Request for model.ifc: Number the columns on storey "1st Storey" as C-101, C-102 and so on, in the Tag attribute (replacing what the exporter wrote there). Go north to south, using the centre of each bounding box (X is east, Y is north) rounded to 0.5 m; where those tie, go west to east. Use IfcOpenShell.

First a look at what the model holds.

```python
import ifcopenshell
import ifcopenshell.util.element
import ifcopenshell.util.placement

model = ifcopenshell.open("model.ifc")
print(model.schema)
storey = next(s for s in model.by_type("IfcBuildingStorey") if s.Name == "1st Storey")
columns = [e for e in ifcopenshell.util.element.get_decomposition(storey) if e.is_a("IfcColumn")]
for e in sorted(columns, key=lambda e: e.id()):
    origin = ifcopenshell.util.placement.get_local_placement(e.ObjectPlacement)[:3, 3]
    print(e.id(), e.Tag, e.Name, origin.round(2) + 0.0, sep=" | ")
```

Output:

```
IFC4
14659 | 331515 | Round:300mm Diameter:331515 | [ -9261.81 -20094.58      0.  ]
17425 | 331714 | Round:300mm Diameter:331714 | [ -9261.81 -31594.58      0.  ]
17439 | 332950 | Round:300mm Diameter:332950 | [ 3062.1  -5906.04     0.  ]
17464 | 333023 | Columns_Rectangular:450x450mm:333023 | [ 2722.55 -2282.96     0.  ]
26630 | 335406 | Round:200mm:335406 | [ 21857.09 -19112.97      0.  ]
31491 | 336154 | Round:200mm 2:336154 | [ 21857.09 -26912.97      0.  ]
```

```python
import ifcopenshell
import ifcopenshell.geom
import ifcopenshell.util.element
import ifcopenshell.util.shape

model = ifcopenshell.open("model.ifc")
settings = ifcopenshell.geom.settings()
settings.set("use-world-coords", True)


def centre(element):
    shape = ifcopenshell.geom.create_shape(settings, element)
    return ifcopenshell.util.shape.get_bbox_centroid(shape.geometry)


storey = next(s for s in model.by_type("IfcBuildingStorey") if s.Name == "1st Storey")
columns = [e for e in ifcopenshell.util.element.get_decomposition(storey) if e.is_a("IfcColumn")]

# Insertion points can sit at a corner or the storey origin, so sort by the geometry (in metres).
centres = {e: centre(e) for e in columns}
columns.sort(key=lambda e: (-round(centres[e][1] / 0.5), centres[e][0]))

for i, e in enumerate(columns, start=1):
    number = f"C-1{i:02d}"
    e.Tag = number
    print(e.id(), number)

model.write("model_updated.ifc")
```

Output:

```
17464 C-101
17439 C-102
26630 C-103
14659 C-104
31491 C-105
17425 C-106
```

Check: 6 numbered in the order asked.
